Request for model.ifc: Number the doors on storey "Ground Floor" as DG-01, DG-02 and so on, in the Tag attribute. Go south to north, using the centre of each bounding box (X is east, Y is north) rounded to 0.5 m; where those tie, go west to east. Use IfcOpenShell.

First a look at what the model holds.

```python
import ifcopenshell
import ifcopenshell.util.element
import ifcopenshell.util.placement

model = ifcopenshell.open("model.ifc")
print(model.schema)
storey = next(s for s in model.by_type("IfcBuildingStorey") if s.Name == "Ground Floor")
doors = [e for e in ifcopenshell.util.element.get_decomposition(storey) if e.is_a("IfcDoor")]
for e in sorted(doors, key=lambda e: e.id()):
    origin = ifcopenshell.util.placement.get_local_placement(e.ObjectPlacement)[:3, 3]
    print(e.id(), e.Tag, e.Name, origin.round(2) + 0.0, sep=" | ")
```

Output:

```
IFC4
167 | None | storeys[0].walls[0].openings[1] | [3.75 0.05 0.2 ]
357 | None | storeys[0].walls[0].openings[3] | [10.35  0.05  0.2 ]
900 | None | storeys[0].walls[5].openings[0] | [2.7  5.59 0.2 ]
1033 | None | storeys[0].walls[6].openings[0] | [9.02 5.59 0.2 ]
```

```python
import ifcopenshell
import ifcopenshell.geom
import ifcopenshell.util.element
import ifcopenshell.util.shape

model = ifcopenshell.open("model.ifc")
settings = ifcopenshell.geom.settings()
settings.set("use-world-coords", True)


def centre(element):
    shape = ifcopenshell.geom.create_shape(settings, element)
    return ifcopenshell.util.shape.get_bbox_centroid(shape.geometry)


storey = next(s for s in model.by_type("IfcBuildingStorey") if s.Name == "Ground Floor")
doors = [e for e in ifcopenshell.util.element.get_decomposition(storey) if e.is_a("IfcDoor")]

# Insertion points can sit at a corner or the storey origin, so sort by the geometry (in metres).
centres = {e: centre(e) for e in doors}
doors.sort(key=lambda e: (round(centres[e][1] / 0.5), centres[e][0]))

for i, e in enumerate(doors, start=1):
    number = f"DG-{i:02d}"
    e.Tag = number
    print(e.id(), number)

model.write("model_v2.ifc")
```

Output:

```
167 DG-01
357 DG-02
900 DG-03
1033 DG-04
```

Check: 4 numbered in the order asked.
